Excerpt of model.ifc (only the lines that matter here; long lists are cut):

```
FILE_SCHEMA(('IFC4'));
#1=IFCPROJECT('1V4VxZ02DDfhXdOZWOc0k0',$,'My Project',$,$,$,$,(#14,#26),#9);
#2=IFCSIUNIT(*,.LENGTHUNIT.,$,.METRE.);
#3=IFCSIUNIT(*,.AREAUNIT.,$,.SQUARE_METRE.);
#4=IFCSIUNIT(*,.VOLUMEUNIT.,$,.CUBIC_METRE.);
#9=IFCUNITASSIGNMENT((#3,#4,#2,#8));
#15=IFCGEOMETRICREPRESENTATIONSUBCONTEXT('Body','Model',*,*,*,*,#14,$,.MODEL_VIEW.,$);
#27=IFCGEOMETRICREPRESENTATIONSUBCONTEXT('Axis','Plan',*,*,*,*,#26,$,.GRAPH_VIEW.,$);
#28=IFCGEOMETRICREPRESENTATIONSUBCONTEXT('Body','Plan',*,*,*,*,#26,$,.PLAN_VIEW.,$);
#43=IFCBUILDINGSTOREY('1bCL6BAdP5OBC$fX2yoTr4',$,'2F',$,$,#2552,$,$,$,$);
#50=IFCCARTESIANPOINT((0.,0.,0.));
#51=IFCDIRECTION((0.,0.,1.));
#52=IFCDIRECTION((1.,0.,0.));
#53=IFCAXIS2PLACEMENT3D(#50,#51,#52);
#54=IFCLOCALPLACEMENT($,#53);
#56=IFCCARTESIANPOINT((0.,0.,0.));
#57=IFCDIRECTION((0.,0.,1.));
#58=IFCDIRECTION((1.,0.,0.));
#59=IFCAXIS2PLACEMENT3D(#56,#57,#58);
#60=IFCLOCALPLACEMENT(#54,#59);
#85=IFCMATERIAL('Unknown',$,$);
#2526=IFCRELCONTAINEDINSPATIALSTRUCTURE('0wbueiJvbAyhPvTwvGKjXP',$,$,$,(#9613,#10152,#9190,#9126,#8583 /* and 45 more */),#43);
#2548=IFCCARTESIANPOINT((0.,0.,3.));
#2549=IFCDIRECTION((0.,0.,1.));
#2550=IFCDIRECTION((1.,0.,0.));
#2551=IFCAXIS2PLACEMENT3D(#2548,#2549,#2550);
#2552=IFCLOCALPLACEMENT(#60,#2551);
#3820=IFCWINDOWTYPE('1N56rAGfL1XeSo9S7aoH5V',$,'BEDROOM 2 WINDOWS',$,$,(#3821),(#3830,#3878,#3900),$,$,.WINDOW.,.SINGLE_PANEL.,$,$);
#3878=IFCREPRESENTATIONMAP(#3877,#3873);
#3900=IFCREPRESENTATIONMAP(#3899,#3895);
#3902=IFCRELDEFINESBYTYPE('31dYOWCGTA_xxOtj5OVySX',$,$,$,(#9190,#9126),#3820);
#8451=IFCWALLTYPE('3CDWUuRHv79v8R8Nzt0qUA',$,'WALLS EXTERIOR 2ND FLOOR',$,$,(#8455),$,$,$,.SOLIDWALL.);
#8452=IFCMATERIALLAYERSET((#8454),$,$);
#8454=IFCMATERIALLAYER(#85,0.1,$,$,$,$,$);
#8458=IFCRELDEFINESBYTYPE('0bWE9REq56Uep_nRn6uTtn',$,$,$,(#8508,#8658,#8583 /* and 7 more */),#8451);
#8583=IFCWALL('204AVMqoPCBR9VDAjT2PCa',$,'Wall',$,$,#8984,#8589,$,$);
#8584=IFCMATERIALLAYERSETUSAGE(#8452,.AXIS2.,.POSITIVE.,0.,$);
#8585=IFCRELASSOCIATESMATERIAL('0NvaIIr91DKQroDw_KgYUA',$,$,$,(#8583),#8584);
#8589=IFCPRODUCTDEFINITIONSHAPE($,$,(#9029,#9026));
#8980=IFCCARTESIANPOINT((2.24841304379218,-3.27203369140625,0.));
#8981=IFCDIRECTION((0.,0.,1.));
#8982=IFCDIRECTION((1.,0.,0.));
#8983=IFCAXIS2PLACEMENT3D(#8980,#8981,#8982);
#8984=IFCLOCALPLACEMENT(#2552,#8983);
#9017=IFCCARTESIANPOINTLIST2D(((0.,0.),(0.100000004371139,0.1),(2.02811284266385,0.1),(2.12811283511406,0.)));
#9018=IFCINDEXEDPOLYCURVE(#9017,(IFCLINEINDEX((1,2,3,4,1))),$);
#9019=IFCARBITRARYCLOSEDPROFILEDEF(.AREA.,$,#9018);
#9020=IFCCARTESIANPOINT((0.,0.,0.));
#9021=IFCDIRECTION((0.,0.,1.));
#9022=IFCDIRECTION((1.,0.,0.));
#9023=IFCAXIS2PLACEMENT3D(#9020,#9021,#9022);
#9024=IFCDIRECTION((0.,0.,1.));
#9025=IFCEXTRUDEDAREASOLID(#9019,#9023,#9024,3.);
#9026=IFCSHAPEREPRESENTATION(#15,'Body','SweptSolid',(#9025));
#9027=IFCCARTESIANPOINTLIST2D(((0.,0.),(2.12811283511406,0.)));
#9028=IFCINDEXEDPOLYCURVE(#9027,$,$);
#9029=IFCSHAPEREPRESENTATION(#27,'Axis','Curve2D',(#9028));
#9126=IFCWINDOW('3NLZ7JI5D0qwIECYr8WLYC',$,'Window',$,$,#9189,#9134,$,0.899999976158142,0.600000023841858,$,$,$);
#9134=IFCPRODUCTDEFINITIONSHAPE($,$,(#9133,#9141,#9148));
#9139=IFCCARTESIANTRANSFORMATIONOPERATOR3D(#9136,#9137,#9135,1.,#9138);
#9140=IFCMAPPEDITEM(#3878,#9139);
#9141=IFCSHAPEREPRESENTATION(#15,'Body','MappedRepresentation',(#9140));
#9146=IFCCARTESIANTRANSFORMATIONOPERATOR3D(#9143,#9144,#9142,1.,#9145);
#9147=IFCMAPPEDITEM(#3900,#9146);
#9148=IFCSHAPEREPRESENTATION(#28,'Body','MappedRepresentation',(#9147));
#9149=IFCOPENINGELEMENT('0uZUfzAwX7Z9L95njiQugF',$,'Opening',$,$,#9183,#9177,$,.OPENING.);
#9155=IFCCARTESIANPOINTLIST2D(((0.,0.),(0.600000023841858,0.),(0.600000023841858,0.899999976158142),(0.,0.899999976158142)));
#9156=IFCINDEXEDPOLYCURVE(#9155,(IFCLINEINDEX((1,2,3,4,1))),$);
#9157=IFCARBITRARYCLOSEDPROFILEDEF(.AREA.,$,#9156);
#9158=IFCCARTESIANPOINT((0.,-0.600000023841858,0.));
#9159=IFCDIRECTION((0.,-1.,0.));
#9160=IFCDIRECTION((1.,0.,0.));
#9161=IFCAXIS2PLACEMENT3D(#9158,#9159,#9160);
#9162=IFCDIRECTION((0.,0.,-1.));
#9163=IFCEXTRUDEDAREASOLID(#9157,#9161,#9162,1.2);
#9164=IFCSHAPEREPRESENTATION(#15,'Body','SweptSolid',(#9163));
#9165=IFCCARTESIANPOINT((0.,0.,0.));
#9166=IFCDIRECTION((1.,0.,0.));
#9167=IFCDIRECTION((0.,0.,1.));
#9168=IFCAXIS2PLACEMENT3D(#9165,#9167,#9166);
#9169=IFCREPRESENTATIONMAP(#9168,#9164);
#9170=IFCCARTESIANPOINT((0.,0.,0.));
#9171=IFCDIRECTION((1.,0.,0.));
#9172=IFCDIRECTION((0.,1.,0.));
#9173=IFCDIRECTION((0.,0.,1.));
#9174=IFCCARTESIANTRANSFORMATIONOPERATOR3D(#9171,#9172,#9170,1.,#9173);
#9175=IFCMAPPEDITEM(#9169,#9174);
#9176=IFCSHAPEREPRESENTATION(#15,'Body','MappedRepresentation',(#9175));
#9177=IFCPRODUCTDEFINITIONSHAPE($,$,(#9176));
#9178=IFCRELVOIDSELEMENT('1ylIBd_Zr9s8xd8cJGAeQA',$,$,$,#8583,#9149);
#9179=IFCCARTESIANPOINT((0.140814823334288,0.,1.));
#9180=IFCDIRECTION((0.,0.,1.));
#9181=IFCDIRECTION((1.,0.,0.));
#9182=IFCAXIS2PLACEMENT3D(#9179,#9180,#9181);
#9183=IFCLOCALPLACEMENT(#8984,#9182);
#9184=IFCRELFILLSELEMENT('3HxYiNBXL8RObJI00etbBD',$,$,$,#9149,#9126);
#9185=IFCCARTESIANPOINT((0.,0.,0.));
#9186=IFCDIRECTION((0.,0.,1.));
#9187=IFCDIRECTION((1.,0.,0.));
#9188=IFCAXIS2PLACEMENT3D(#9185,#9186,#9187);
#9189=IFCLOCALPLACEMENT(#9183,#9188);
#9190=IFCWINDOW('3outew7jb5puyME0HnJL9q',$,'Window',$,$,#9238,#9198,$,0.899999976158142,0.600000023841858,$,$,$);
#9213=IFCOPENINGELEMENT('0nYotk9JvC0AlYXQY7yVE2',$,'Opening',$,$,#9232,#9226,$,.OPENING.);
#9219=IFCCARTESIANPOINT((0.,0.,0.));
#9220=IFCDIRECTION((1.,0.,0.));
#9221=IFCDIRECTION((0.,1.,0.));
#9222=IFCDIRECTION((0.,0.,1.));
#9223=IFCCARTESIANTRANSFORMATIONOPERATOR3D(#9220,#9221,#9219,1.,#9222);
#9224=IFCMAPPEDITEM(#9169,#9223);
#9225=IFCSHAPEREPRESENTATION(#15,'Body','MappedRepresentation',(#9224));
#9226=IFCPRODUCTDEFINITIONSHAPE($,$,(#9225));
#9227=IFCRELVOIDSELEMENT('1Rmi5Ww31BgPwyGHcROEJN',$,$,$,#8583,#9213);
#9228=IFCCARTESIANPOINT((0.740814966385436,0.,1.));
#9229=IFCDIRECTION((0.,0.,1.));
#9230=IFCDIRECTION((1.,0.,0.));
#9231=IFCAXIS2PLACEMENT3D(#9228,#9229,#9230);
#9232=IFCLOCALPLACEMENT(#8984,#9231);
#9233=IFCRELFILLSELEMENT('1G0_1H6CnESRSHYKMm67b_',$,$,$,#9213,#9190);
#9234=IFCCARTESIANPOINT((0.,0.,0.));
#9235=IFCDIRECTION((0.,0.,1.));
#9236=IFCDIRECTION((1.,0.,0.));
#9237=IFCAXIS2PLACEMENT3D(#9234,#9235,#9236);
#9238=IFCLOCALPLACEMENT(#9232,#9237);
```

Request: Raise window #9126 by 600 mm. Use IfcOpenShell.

```python
import numpy as np
import ifcopenshell
import ifcopenshell.api.geometry
import ifcopenshell.util.placement
import ifcopenshell.util.unit

model = ifcopenshell.open("model.ifc")
unit_scale = ifcopenshell.util.unit.calculate_unit_scale(model)

window = model.by_guid("3NLZ7JI5D0qwIECYr8WLYC")
opening = window.FillsVoids[0].RelatingOpeningElement
dz = 0.6

shift = np.array([0.0, 0.0, dz])
# The window is placed relative to its opening, so it follows when the opening moves.
matrix = ifcopenshell.util.placement.get_local_placement(opening.ObjectPlacement)
matrix[:3, 3] += shift
ifcopenshell.api.geometry.edit_object_placement(
    model, product=opening, matrix=matrix, is_si=False, should_transform_children=True
)

print(f"moved by {dz * unit_scale:+.3f} m")

model.write("model_v2.ifc")
```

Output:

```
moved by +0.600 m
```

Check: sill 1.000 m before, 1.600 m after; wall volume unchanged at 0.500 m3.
